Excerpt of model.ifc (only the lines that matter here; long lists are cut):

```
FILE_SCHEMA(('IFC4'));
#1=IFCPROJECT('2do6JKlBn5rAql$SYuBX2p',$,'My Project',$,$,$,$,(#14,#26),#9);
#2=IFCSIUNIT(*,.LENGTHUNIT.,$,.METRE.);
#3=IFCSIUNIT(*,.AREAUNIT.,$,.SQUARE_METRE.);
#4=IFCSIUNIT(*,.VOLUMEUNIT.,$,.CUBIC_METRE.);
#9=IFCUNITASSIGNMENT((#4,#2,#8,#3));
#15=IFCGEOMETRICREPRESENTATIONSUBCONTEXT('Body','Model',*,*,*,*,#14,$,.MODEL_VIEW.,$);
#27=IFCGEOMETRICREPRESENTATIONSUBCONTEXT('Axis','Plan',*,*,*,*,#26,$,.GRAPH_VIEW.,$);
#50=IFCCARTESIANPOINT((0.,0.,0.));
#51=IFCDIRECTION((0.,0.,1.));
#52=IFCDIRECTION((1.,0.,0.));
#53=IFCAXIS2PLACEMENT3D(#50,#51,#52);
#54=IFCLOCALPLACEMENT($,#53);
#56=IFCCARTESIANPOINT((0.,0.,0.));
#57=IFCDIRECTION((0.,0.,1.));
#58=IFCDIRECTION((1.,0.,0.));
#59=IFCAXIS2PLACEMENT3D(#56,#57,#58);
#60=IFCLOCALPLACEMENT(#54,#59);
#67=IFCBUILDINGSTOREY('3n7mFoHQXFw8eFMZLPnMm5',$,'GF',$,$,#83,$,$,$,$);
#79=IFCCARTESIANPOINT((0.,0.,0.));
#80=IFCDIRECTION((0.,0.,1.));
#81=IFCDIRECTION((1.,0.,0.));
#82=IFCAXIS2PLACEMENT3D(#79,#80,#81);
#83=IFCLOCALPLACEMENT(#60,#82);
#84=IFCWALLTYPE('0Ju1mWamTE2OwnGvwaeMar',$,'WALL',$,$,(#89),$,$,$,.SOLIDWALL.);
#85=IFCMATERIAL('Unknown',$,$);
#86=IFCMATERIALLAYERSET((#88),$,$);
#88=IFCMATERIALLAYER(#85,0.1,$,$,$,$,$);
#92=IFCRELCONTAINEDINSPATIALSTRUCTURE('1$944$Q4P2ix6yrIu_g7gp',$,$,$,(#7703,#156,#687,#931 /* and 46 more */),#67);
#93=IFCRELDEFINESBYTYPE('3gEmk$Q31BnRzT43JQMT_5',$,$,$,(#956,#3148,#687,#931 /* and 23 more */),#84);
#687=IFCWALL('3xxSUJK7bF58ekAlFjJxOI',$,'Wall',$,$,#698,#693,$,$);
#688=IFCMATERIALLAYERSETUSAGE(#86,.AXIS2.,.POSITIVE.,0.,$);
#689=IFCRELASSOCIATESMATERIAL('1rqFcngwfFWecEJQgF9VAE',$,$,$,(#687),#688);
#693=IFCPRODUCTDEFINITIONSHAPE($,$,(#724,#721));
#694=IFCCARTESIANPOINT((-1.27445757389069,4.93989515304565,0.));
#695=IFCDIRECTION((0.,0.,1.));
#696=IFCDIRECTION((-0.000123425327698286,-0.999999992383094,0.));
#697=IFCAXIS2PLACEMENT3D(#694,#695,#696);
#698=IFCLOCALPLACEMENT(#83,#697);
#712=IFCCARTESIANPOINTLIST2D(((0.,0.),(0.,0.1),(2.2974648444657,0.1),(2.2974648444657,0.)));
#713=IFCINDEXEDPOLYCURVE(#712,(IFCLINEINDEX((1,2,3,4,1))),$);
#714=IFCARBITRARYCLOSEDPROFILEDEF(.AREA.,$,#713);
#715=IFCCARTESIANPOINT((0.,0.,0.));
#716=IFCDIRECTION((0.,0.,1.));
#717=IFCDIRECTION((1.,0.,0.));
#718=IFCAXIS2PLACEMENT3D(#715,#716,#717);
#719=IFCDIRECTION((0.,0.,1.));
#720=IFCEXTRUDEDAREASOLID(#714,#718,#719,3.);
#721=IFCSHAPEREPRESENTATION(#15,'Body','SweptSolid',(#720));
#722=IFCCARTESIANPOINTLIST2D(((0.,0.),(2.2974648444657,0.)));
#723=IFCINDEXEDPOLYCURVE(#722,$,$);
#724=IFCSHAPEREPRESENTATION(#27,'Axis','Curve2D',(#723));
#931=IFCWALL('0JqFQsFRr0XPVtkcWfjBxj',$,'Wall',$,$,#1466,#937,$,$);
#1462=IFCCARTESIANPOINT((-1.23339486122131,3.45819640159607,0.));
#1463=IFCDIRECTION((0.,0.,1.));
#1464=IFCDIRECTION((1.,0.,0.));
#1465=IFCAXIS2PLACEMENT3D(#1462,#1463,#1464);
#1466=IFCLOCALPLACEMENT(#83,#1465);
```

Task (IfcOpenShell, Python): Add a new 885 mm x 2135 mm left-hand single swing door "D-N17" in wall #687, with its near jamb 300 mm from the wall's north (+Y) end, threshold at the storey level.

```python
import numpy as np
import ifcopenshell
import ifcopenshell.api.feature
import ifcopenshell.api.geometry
import ifcopenshell.api.root
import ifcopenshell.api.spatial
import ifcopenshell.geom
import ifcopenshell.util.element
import ifcopenshell.util.placement
import ifcopenshell.util.representation
import ifcopenshell.util.shape
import ifcopenshell.util.unit

model = ifcopenshell.open("model.ifc")
unit_scale = ifcopenshell.util.unit.calculate_unit_scale(model)
settings = ifcopenshell.geom.settings()


def volume(element):
    """Net volume in cubic metres, openings subtracted."""
    shape = ifcopenshell.geom.create_shape(settings, element)
    return ifcopenshell.util.shape.get_volume(shape.geometry)


wall = model.by_guid("3xxSUJK7bF58ekAlFjJxOI")
storey = ifcopenshell.util.element.get_container(wall, ifc_class="IfcBuildingStorey")
context = ifcopenshell.util.representation.get_context(model, "Model", "Body", "MODEL_VIEW")
before = volume(wall)

width, height, from_end, sill = 0.885, 2.135, 0.3, 0.0  # metres

# The wall runs along its own X axis, and the end named is its -X end.
wall_shape = ifcopenshell.geom.create_shape(settings, wall)
x, y, z = ifcopenshell.util.shape.get_vertices(wall_shape.geometry).T
start = x.min() + from_end
face, thickness = float(y.min()), float(y.max() - y.min())
wall_matrix = ifcopenshell.util.placement.get_local_placement(wall.ObjectPlacement)
level = ifcopenshell.util.placement.get_local_placement(storey.ObjectPlacement)[2, 3]


def in_wall(x, y):
    """Placement at x, y metres in the wall's axes, at sill height."""
    matrix = wall_matrix.copy()
    matrix[:, 3] = wall_matrix @ np.array([x / unit_scale, y / unit_scale, 0.0, 1.0])
    matrix[2, 3] = level + sill / unit_scale
    return matrix


# Opening: a box that overshoots both wall faces by 50 mm.
opening = ifcopenshell.api.root.create_entity(model, ifc_class="IfcOpeningElement", predefined_type="OPENING")
box = ifcopenshell.api.geometry.add_wall_representation(
    model, context=context, length=width, height=height, thickness=thickness + 0.1
)
ifcopenshell.api.geometry.assign_representation(model, product=opening, representation=box)
ifcopenshell.api.geometry.edit_object_placement(model, product=opening, matrix=in_wall(start, face - 0.05), is_si=False)
ifcopenshell.api.feature.add_feature(model, feature=opening, element=wall)

door = ifcopenshell.api.root.create_entity(model, ifc_class="IfcDoor", name="D-N17", predefined_type="DOOR")
door.OverallWidth, door.OverallHeight = width / unit_scale, height / unit_scale
door.OperationType = "SINGLE_SWING_LEFT"
body = ifcopenshell.api.geometry.add_door_representation(
    model,
    context=context,
    overall_width=door.OverallWidth,
    overall_height=door.OverallHeight,
    operation_type="SINGLE_SWING_LEFT",
    lining_properties={"LiningDepth": thickness / unit_scale, "ThresholdDepth": thickness / unit_scale},
)
ifcopenshell.api.geometry.assign_representation(model, product=door, representation=body)
ifcopenshell.api.spatial.assign_container(model, products=[door], relating_structure=storey)
ifcopenshell.api.feature.add_filling(model, opening=opening, element=door)

# The lining spans the wall, so the door starts at the wall face.
ifcopenshell.api.geometry.edit_object_placement(model, product=door, matrix=in_wall(start, face), is_si=False)

after = volume(wall)

print(f"wall volume {before:.3f} -> {after:.3f} m3")

model.write("model-out.ifc")
```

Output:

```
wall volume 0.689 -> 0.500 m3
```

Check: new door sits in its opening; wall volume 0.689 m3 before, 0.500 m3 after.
